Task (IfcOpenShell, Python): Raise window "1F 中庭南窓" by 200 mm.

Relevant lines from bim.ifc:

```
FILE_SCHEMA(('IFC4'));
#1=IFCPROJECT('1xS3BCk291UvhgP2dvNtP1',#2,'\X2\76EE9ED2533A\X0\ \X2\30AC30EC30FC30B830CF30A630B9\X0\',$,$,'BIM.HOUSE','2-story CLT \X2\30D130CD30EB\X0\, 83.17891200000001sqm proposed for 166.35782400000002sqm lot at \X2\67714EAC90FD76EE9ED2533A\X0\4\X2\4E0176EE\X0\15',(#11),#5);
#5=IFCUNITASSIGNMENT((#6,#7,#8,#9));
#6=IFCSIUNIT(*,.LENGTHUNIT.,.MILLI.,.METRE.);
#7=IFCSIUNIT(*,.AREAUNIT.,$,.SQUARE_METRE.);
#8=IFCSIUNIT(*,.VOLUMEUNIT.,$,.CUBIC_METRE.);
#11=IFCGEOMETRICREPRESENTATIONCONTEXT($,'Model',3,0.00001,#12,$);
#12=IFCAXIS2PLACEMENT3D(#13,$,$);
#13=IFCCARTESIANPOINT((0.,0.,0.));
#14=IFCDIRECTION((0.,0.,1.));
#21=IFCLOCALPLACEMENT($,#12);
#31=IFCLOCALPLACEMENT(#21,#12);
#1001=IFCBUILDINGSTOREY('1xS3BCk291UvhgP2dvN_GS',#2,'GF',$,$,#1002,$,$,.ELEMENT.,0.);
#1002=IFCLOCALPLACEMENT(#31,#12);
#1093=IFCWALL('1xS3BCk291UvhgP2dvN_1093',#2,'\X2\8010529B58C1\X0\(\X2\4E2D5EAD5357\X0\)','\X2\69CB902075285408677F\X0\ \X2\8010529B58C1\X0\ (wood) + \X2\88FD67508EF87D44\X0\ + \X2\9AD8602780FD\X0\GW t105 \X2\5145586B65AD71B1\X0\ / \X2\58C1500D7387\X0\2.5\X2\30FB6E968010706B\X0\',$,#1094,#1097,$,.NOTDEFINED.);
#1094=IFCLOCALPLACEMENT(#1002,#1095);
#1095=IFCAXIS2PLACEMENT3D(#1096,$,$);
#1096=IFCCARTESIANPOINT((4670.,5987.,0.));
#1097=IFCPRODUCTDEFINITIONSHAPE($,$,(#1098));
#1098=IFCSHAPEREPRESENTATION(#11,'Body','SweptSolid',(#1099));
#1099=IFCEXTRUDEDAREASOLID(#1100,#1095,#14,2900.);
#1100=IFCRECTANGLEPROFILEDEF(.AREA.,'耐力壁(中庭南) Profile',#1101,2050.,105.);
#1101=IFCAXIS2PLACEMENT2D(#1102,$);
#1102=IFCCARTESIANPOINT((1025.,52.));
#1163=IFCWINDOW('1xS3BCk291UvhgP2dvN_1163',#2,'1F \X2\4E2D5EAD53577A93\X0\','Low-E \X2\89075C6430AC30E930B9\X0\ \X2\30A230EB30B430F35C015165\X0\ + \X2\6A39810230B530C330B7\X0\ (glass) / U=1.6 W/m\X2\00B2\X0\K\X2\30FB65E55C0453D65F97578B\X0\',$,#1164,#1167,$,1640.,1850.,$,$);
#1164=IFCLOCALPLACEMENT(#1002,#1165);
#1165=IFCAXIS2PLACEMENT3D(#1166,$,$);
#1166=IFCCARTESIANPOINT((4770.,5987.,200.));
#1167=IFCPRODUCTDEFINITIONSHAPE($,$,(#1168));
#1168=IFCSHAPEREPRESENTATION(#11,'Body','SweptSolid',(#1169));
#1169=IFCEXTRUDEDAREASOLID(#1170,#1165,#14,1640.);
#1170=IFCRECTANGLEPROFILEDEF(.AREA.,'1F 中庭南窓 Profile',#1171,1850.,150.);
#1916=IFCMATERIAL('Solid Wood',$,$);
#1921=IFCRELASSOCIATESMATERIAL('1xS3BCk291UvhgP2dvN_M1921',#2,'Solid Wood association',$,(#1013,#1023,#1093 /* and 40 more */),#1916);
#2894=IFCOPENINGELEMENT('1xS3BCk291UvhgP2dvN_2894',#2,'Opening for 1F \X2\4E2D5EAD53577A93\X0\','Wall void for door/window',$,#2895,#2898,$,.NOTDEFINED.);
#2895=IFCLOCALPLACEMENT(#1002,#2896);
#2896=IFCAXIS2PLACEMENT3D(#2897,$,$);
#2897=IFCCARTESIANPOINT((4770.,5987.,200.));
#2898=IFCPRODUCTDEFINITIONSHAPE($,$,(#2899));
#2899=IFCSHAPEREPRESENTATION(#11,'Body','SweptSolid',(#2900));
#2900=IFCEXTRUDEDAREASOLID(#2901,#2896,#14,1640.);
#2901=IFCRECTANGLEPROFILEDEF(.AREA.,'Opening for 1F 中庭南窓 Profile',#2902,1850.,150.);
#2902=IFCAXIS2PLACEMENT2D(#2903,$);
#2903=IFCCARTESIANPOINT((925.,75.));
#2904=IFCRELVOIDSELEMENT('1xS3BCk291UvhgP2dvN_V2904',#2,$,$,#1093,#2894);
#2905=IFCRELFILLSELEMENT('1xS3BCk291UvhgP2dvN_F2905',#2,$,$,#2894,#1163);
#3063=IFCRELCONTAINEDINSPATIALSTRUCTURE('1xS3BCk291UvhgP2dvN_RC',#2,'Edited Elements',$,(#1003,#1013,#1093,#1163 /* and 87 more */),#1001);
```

```python
import numpy as np
import ifcopenshell
import ifcopenshell.api.geometry
import ifcopenshell.util.placement
import ifcopenshell.util.unit

model = ifcopenshell.open("bim.ifc")
unit_scale = ifcopenshell.util.unit.calculate_unit_scale(model)

window = model.by_guid("1xS3BCk291UvhgP2dvN_1163")
opening = window.FillsVoids[0].RelatingOpeningElement
dz = 200.0

shift = np.array([0.0, 0.0, dz])
# The window is not placed relative to its opening, so move both.
for product in (opening, window):
    matrix = ifcopenshell.util.placement.get_local_placement(product.ObjectPlacement)
    matrix[:3, 3] += shift
    ifcopenshell.api.geometry.edit_object_placement(model, product=product, matrix=matrix, is_si=False)

print(f"moved by {dz * unit_scale:+.3f} m")

model.write("bim_updated.ifc")
```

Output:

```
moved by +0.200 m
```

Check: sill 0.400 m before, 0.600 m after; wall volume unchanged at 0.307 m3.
